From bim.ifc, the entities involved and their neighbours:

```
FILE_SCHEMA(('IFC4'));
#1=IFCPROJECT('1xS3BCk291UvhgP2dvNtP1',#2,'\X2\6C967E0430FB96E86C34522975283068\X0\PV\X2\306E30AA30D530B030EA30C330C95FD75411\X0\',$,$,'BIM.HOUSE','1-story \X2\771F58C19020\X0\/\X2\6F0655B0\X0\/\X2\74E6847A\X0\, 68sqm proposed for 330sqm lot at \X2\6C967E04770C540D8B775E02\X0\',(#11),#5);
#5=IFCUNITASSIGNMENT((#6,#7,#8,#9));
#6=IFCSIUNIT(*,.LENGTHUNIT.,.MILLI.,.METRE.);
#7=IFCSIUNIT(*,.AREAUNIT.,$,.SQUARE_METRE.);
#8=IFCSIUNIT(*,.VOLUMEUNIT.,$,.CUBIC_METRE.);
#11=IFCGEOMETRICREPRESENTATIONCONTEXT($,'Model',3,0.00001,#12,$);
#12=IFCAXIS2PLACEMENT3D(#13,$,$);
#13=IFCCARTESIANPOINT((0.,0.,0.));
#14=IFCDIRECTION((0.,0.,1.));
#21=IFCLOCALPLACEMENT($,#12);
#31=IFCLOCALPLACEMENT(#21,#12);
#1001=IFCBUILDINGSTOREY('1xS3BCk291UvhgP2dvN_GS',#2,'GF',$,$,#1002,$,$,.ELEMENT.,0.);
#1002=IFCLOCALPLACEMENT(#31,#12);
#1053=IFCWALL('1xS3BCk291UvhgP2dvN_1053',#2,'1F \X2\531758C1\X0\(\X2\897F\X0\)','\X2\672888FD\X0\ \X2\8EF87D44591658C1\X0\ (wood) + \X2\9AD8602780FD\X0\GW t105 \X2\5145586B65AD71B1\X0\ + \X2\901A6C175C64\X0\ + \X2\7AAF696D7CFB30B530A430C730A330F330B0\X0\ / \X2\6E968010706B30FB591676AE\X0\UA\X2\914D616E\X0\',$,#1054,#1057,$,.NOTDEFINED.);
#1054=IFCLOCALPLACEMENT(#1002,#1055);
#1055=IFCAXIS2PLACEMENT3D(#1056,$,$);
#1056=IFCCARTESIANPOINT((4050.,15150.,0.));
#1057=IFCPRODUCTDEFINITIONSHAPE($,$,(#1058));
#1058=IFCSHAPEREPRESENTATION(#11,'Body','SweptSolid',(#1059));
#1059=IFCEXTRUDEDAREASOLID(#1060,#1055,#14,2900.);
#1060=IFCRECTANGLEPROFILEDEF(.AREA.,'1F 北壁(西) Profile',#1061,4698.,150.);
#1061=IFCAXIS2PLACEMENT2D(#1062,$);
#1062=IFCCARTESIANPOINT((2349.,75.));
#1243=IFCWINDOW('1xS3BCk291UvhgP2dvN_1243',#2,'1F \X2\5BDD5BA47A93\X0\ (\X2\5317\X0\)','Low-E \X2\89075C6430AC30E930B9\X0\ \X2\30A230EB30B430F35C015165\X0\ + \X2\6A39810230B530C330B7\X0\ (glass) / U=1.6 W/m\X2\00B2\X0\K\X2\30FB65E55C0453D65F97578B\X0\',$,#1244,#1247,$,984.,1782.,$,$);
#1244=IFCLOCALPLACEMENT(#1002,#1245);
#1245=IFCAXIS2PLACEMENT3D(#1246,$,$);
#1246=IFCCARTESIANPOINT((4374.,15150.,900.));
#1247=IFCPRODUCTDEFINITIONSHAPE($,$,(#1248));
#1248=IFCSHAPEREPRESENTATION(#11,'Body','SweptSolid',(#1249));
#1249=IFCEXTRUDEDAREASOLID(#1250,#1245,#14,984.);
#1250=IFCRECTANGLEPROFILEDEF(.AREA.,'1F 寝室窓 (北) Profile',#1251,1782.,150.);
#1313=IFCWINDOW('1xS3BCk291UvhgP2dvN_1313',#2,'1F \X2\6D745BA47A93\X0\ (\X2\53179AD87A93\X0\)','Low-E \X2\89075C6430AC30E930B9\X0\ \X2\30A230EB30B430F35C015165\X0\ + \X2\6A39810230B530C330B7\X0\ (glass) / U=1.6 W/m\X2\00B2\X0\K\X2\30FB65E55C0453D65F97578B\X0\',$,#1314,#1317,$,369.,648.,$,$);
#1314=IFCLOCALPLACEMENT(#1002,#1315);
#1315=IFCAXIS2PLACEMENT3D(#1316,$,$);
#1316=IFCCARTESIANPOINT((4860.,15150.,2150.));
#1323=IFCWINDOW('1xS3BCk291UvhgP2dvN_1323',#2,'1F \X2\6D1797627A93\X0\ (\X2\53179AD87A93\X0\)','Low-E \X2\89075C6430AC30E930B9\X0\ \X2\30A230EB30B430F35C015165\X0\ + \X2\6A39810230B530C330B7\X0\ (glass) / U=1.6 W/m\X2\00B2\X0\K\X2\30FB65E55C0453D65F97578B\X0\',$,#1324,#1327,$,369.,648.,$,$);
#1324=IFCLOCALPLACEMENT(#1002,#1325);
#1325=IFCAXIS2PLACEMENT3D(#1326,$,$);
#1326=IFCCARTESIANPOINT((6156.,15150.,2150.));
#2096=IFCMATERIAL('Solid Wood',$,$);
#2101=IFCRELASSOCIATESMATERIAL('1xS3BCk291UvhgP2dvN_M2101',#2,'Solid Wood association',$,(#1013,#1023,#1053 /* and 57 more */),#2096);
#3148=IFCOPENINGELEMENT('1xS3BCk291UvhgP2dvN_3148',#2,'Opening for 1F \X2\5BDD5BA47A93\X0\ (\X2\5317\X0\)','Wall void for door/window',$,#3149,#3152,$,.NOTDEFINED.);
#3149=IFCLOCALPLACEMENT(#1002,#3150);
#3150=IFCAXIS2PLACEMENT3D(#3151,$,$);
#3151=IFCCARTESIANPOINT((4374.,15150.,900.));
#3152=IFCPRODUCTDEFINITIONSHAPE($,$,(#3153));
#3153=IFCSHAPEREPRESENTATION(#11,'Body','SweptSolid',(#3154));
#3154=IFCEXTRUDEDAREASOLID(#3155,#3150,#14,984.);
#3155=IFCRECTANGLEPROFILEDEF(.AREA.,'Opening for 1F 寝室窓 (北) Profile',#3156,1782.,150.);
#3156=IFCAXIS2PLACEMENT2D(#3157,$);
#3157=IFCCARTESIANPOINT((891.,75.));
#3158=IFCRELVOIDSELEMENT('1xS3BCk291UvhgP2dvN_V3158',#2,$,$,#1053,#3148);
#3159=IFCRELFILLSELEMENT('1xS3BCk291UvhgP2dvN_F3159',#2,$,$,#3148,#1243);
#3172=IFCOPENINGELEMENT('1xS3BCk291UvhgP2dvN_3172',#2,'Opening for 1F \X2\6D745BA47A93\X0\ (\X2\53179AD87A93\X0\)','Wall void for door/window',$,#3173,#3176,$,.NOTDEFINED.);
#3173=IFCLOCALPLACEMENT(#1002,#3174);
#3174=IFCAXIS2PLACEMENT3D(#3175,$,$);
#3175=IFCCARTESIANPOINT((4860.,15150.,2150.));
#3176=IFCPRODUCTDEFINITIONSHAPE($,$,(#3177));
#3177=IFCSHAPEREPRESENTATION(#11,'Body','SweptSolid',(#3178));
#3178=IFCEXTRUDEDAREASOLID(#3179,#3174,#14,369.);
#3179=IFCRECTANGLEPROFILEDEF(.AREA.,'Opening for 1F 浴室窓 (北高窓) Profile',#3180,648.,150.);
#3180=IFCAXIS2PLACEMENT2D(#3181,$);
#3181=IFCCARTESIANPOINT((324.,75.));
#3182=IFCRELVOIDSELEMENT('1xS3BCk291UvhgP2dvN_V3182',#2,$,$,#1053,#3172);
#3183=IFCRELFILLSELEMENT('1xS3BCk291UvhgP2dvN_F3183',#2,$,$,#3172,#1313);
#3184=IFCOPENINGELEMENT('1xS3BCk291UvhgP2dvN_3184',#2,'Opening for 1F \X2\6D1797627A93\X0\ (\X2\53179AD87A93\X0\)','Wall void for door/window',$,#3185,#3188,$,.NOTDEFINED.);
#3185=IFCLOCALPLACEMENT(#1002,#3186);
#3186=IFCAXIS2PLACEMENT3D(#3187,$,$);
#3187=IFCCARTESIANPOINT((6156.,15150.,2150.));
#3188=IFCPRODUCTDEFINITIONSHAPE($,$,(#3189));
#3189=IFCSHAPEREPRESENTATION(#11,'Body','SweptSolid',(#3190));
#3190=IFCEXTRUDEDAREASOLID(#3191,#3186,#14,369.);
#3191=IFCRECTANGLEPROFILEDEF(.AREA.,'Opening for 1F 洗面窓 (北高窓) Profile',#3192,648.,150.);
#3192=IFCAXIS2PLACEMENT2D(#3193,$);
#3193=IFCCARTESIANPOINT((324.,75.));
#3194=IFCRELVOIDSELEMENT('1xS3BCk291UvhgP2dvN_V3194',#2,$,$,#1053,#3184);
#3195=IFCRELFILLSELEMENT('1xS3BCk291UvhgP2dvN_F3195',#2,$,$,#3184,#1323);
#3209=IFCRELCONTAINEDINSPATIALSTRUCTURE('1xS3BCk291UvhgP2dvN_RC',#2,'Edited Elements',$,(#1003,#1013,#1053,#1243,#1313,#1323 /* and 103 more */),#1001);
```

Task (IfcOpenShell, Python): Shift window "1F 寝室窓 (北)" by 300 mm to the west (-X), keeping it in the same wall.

```python
import ifcopenshell
import ifcopenshell.api.geometry
import ifcopenshell.util.placement
import ifcopenshell.util.unit

model = ifcopenshell.open("bim.ifc")
unit_scale = ifcopenshell.util.unit.calculate_unit_scale(model)

window = model.by_guid("1xS3BCk291UvhgP2dvN_1243")
opening = window.FillsVoids[0].RelatingOpeningElement
wall = opening.VoidsElements[0].RelatingBuildingElement

wall_matrix = ifcopenshell.util.placement.get_local_placement(wall.ObjectPlacement)
shift = wall_matrix[:3, 0] * -0.3 / unit_scale
before = ifcopenshell.util.placement.get_local_placement(window.ObjectPlacement)[:3, 3].copy()

# The window is not placed relative to its opening, so move both.
for product in (opening, window):
    matrix = ifcopenshell.util.placement.get_local_placement(product.ObjectPlacement)
    matrix[:3, 3] += shift
    ifcopenshell.api.geometry.edit_object_placement(model, product=product, matrix=matrix, is_si=False)

after = ifcopenshell.util.placement.get_local_placement(window.ObjectPlacement)[:3, 3]
print("window moved by", (after - before).round(3) + 0.0)

model.write("bim_edited.ifc")
```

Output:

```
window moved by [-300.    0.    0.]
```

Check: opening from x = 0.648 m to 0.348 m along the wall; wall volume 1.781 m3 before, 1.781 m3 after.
